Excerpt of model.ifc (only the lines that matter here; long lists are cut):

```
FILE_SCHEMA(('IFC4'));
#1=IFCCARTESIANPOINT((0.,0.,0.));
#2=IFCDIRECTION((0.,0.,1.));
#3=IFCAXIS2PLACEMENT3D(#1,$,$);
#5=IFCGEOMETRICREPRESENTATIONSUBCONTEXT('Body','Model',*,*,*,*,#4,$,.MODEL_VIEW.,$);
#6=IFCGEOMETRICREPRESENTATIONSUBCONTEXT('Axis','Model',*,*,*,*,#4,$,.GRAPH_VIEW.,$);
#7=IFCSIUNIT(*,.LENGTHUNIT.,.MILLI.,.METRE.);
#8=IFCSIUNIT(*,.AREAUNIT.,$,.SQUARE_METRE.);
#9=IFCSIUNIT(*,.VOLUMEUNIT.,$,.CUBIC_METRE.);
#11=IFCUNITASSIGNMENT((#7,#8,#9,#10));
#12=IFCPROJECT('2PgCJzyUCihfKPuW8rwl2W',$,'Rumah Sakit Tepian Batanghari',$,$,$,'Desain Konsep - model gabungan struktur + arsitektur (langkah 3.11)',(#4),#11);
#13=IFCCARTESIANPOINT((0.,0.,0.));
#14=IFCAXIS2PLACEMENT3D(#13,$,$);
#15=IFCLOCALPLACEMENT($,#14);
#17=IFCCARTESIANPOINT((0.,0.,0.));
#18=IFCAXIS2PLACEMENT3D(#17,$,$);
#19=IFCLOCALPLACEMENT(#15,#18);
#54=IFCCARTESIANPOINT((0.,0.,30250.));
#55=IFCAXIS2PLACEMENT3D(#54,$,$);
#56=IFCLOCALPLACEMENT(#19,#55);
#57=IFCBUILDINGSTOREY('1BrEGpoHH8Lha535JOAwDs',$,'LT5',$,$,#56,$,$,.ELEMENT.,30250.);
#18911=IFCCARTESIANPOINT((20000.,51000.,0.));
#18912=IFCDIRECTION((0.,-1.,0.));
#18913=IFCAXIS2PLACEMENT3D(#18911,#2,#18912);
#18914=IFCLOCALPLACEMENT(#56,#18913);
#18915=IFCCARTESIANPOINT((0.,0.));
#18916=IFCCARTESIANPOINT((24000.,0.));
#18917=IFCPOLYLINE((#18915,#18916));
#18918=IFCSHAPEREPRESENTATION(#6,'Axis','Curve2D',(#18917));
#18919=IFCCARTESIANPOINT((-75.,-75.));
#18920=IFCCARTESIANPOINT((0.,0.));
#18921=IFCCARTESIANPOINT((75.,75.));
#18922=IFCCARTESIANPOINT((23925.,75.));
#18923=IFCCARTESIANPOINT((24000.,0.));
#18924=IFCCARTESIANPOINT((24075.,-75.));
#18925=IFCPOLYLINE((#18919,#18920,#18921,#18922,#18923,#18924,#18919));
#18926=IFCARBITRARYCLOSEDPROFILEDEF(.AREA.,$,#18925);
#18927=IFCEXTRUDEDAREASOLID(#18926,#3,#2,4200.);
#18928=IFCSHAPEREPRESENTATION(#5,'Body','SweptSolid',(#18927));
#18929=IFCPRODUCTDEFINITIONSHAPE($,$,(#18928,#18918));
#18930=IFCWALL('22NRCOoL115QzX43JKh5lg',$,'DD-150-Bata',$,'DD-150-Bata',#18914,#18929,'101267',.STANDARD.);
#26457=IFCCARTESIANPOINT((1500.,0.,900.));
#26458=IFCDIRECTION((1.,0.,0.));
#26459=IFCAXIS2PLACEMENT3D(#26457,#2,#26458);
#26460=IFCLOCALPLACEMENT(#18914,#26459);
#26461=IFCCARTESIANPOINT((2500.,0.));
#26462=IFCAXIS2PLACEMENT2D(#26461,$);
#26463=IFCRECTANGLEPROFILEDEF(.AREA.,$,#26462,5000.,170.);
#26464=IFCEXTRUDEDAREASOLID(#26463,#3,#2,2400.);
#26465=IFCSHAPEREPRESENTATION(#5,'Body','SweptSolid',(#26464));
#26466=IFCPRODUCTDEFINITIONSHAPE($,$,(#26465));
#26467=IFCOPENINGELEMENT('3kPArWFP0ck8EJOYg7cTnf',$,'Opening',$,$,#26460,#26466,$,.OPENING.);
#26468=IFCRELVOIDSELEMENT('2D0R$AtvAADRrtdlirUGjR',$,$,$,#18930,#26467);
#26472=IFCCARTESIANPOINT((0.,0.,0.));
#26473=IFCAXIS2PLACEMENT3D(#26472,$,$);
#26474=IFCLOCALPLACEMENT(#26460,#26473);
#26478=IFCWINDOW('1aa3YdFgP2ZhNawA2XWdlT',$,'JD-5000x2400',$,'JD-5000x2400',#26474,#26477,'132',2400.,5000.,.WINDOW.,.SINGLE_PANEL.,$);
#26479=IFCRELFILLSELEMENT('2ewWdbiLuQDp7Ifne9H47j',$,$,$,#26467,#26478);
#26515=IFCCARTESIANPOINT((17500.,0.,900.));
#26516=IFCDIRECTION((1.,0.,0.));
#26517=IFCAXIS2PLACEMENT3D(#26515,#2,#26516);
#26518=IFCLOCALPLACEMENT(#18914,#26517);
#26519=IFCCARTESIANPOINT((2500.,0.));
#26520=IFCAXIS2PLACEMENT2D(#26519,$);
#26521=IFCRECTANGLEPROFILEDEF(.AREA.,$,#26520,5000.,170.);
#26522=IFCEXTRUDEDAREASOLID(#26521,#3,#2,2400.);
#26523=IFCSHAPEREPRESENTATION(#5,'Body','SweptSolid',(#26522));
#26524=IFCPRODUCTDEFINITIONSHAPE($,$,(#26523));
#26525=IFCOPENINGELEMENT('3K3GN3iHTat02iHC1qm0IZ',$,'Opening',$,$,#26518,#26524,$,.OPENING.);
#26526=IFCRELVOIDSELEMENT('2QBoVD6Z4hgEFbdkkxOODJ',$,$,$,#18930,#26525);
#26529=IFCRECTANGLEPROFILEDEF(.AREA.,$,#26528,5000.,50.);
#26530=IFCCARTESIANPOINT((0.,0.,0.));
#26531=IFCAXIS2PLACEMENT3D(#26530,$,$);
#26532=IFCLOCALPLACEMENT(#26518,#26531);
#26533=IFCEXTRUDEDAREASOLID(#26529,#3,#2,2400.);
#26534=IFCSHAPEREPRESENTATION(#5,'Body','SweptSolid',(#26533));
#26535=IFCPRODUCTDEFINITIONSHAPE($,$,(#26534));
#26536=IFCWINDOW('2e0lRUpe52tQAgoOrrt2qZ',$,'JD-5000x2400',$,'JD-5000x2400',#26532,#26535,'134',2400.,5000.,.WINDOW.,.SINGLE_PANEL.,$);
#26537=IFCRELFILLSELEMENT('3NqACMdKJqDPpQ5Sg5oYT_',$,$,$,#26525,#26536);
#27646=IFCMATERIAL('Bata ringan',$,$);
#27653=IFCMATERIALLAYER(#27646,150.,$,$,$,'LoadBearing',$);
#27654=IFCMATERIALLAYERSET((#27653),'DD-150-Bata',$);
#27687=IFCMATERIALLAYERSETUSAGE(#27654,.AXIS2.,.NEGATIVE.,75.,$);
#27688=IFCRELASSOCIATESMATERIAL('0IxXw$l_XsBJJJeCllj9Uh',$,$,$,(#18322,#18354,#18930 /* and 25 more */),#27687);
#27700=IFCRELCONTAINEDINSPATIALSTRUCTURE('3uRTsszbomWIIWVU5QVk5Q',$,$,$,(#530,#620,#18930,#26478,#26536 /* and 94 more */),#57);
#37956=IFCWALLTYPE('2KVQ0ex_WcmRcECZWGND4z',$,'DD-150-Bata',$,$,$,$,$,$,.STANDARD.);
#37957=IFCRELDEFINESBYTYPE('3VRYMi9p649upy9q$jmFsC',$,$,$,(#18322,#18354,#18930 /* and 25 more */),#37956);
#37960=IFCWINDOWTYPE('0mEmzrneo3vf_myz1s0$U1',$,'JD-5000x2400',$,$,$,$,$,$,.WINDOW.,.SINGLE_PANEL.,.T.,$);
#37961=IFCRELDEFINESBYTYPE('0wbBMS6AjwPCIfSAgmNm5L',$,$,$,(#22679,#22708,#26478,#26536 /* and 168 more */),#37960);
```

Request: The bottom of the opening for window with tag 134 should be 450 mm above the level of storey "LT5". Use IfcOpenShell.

```python
import numpy as np
import ifcopenshell
import ifcopenshell.api.geometry
import ifcopenshell.geom
import ifcopenshell.util.element
import ifcopenshell.util.placement
import ifcopenshell.util.shape
import ifcopenshell.util.unit

model = ifcopenshell.open("model.ifc")
unit_scale = ifcopenshell.util.unit.calculate_unit_scale(model)

window = model.by_guid("2e0lRUpe52tQAgoOrrt2qZ")
opening = window.FillsVoids[0].RelatingOpeningElement
storey = ifcopenshell.util.element.get_container(window, ifc_class="IfcBuildingStorey")
level = ifcopenshell.util.placement.get_local_placement(storey.ObjectPlacement)[2, 3]

# The opening's origin need not be at the sill, so measure its lowest point.
shape = ifcopenshell.geom.create_shape(ifcopenshell.geom.settings(), opening)
bottom = ifcopenshell.util.shape.get_shape_bottom_elevation(shape, shape.geometry) / unit_scale
dz = level + 450.0 - bottom

shift = np.array([0.0, 0.0, dz])
# The window is placed relative to its opening, so it follows when the opening moves.
matrix = ifcopenshell.util.placement.get_local_placement(opening.ObjectPlacement)
matrix[:3, 3] += shift
ifcopenshell.api.geometry.edit_object_placement(
    model, product=opening, matrix=matrix, is_si=False, should_transform_children=True
)

print(f"moved by {dz * unit_scale:+.3f} m")

model.write("model_edited.ifc")
```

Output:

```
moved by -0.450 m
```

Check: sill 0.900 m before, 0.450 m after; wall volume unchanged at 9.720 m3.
